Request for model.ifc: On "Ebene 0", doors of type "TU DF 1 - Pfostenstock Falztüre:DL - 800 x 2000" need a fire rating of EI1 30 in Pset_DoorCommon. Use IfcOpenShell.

First a look at what the model holds.

```python
import ifcopenshell
import ifcopenshell.util.element

model = ifcopenshell.open("model.ifc")
print(model.schema)
storey = next(s for s in model.by_type("IfcBuildingStorey") if s.Name == "Ebene 0")
doors = [e for e in ifcopenshell.util.element.get_decomposition(storey) if e.is_a("IfcDoor")]
seen = {}
for e in doors:
    element_type = ifcopenshell.util.element.get_type(e)
    key = (element_type.Name if element_type != e and element_type else None, ifcopenshell.util.element.get_pset(e, "Pset_DoorCommon", "FireRating"))
    seen[key] = seen.get(key, 0) + 1
for (name, value), count in sorted(seen.items(), key=str):
    print(count, "x", name, "|", value)
```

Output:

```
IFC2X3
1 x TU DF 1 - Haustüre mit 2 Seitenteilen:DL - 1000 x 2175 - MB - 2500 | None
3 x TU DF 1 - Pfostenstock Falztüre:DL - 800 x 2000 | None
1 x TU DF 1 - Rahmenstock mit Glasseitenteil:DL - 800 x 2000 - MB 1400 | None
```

```python
import ifcopenshell
import ifcopenshell.api.pset
import ifcopenshell.util.element

model = ifcopenshell.open("model.ifc")

storey = next(s for s in model.by_type("IfcBuildingStorey") if s.Name == "Ebene 0")
doors = [e for e in ifcopenshell.util.element.get_decomposition(storey) if e.is_a("IfcDoor")]

count = 0
for e in doors:
    element_type = ifcopenshell.util.element.get_type(e)
    if element_type in (None, e) or element_type.Name != "TU DF 1 - Pfostenstock Falztüre:DL - 800 x 2000":
        continue
    # add_pset returns the element's existing set when there is one.
    pset = ifcopenshell.api.pset.add_pset(model, product=e, name="Pset_DoorCommon")
    ifcopenshell.api.pset.edit_pset(model, pset=pset, properties={"FireRating": "EI1 30"})
    count += 1

print(count, "doors updated")

model.write("model_rev.ifc")
```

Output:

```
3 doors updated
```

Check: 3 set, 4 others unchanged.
